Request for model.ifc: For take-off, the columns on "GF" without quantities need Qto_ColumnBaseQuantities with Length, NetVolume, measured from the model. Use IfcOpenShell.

First a look at what the model holds.

```python
import ifcopenshell
import ifcopenshell.util.element
import ifcopenshell.util.unit

model = ifcopenshell.open("model.ifc")
print(model.schema)
for unit_type in ("LENGTHUNIT", "AREAUNIT", "VOLUMEUNIT"):
    print(unit_type, ifcopenshell.util.unit.calculate_unit_scale(model, unit_type))
storey = next(s for s in model.by_type("IfcBuildingStorey") if s.Name == "GF")
columns = [e for e in ifcopenshell.util.element.get_decomposition(storey) if e.is_a("IfcColumn")]
for e in sorted(columns, key=lambda e: e.id()):
    print(e.id(), e.is_a(), e.Name, list(ifcopenshell.util.element.get_psets(e, qtos_only=True)), sep=" | ")
```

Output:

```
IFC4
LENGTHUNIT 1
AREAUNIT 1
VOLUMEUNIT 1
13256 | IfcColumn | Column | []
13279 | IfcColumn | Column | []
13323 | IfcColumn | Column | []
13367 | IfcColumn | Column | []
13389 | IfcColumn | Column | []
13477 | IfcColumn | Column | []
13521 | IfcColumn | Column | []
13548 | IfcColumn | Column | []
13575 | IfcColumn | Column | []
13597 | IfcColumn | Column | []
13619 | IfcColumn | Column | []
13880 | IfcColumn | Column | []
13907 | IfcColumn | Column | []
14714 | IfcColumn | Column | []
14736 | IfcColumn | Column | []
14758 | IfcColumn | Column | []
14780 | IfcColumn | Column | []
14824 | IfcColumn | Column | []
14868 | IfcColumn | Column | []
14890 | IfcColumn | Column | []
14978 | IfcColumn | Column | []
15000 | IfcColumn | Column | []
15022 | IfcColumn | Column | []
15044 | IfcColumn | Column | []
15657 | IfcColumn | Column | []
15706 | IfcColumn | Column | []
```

```python
import ifcopenshell
import ifcopenshell.api.pset
import ifcopenshell.geom
import ifcopenshell.util.element
import ifcopenshell.util.shape
import ifcopenshell.util.unit

model = ifcopenshell.open("model.ifc")
unit_scale = ifcopenshell.util.unit.calculate_unit_scale(model)
volume_scale = ifcopenshell.util.unit.calculate_unit_scale(model, "VOLUMEUNIT")
settings = ifcopenshell.geom.settings()

storey = next(s for s in model.by_type("IfcBuildingStorey") if s.Name == "GF")
columns = [e for e in ifcopenshell.util.element.get_decomposition(storey) if e.is_a("IfcColumn")]

for e in sorted(columns, key=lambda e: e.id()):
    if ifcopenshell.util.element.get_psets(e, qtos_only=True, should_inherit=False):
        continue
    # Geometry comes back in metres, in the element's own axes.
    shape = ifcopenshell.geom.create_shape(settings, e)
    values = {
        "Length": ifcopenshell.util.shape.get_z(shape.geometry) / unit_scale,
        "NetVolume": ifcopenshell.util.shape.get_volume(shape.geometry) / volume_scale,
    }
    qto = ifcopenshell.api.pset.add_qto(model, product=e, name="Qto_ColumnBaseQuantities")
    ifcopenshell.api.pset.edit_qto(model, qto=qto, properties=values)
    print(e.id(), {k: round(v, 3) for k, v in values.items()})

model.write("model_updated.ifc")
```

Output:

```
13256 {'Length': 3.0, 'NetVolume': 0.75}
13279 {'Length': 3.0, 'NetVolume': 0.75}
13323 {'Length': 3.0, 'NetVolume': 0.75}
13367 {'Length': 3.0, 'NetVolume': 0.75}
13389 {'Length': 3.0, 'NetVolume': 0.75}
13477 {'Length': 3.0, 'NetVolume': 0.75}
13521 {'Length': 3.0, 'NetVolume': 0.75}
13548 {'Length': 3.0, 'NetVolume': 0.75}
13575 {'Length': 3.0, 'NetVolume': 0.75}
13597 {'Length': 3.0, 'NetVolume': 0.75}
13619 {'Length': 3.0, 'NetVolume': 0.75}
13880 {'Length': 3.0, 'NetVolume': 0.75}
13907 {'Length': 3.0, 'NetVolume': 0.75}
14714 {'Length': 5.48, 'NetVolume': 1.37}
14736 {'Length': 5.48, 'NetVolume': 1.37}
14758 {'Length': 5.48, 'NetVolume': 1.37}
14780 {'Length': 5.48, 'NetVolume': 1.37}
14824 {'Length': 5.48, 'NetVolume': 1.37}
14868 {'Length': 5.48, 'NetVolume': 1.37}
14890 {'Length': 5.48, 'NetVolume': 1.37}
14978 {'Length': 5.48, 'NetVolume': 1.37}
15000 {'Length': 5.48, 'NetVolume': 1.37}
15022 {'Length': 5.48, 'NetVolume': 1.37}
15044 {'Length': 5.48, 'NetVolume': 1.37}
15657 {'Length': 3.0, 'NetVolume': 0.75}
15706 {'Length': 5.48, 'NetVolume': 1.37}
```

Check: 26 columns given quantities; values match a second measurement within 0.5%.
